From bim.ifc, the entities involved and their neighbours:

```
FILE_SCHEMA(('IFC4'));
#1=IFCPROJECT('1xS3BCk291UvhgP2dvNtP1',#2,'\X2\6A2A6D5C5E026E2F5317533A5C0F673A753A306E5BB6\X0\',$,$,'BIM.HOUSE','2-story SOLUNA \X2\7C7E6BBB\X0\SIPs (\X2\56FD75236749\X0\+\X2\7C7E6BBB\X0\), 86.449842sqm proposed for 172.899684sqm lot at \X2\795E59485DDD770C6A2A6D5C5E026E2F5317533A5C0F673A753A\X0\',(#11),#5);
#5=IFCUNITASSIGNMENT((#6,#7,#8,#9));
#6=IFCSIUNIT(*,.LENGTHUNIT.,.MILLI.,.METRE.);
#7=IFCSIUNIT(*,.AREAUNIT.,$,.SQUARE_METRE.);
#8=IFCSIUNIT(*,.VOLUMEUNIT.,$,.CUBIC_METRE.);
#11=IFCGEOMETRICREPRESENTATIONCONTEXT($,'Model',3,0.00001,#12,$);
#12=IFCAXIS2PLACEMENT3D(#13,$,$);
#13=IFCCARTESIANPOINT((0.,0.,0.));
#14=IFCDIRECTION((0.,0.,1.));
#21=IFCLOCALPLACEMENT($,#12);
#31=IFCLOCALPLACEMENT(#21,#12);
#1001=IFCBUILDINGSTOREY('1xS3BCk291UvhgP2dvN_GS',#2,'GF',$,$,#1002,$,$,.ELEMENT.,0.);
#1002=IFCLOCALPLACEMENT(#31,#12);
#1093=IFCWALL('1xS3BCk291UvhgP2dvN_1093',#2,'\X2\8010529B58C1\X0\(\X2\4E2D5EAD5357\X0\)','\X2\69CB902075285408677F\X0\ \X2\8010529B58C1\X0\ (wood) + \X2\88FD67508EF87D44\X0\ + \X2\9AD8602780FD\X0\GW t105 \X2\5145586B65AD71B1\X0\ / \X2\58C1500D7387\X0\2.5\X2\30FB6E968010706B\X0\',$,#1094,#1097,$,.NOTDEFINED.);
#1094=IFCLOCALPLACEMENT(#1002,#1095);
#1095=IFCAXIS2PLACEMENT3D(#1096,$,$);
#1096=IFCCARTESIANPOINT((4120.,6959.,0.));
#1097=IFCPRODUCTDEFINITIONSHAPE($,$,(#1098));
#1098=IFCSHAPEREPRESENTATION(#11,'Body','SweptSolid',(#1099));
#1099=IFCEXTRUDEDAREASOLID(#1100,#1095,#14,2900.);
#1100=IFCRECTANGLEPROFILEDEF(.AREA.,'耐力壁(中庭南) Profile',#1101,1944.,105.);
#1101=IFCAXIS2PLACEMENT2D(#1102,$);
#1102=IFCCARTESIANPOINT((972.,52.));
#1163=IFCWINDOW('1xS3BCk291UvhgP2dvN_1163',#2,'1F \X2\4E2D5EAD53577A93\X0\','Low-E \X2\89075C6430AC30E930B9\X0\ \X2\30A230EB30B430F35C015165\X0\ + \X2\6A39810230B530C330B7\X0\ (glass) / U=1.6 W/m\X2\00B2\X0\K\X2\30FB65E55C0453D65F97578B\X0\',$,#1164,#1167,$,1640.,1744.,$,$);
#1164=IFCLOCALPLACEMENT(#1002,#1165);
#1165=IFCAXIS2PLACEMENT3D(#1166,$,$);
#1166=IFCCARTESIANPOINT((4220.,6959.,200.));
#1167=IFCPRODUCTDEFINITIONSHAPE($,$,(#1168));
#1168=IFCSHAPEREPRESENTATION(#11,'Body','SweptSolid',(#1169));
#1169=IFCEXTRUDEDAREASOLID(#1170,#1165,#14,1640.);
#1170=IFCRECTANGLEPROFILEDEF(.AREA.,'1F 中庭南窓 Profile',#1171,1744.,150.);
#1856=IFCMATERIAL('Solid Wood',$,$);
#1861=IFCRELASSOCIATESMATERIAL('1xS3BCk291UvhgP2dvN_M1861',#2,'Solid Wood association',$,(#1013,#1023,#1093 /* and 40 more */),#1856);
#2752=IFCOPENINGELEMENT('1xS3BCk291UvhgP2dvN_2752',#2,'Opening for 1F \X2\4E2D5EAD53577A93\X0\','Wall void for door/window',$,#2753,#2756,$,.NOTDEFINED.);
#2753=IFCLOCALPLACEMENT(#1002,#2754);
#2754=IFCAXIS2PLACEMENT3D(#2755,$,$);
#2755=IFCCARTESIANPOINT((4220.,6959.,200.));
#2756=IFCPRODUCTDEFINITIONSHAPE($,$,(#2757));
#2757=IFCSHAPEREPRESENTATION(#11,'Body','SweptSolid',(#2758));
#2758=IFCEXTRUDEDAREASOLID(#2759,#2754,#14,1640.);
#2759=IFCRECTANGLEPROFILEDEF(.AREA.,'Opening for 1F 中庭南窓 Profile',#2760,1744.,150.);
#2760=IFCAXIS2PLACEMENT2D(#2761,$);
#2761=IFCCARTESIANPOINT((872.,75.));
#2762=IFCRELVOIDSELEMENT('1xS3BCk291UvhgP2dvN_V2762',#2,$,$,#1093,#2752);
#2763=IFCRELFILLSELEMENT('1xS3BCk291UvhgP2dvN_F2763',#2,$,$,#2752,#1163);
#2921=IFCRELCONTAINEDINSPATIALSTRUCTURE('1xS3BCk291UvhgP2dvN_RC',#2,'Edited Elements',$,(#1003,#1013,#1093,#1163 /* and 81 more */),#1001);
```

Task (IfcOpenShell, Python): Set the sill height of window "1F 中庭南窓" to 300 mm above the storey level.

```python
import numpy as np
import ifcopenshell
import ifcopenshell.api.geometry
import ifcopenshell.geom
import ifcopenshell.util.element
import ifcopenshell.util.placement
import ifcopenshell.util.shape
import ifcopenshell.util.unit

model = ifcopenshell.open("bim.ifc")
unit_scale = ifcopenshell.util.unit.calculate_unit_scale(model)

window = model.by_id(1163)
opening = window.FillsVoids[0].RelatingOpeningElement
storey = ifcopenshell.util.element.get_container(window, ifc_class="IfcBuildingStorey")
level = ifcopenshell.util.placement.get_local_placement(storey.ObjectPlacement)[2, 3]

# The opening's origin need not be at the sill, so measure its lowest point.
shape = ifcopenshell.geom.create_shape(ifcopenshell.geom.settings(), opening)
bottom = ifcopenshell.util.shape.get_shape_bottom_elevation(shape, shape.geometry) / unit_scale
dz = level + 0.3 / unit_scale - bottom

shift = np.array([0.0, 0.0, dz])
# The window is not placed relative to its opening, so move both.
for product in (opening, window):
    matrix = ifcopenshell.util.placement.get_local_placement(product.ObjectPlacement)
    matrix[:3, 3] += shift
    ifcopenshell.api.geometry.edit_object_placement(model, product=product, matrix=matrix, is_si=False)

print(f"moved by {dz * unit_scale:+.3f} m")

model.write("bim_v2.ifc")
```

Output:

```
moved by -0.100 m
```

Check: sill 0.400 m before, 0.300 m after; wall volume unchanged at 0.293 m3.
